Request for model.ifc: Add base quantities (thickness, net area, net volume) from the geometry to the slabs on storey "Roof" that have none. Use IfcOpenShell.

First a look at what the model holds.

```python
import ifcopenshell
import ifcopenshell.util.element
import ifcopenshell.util.unit

model = ifcopenshell.open("model.ifc")
print(model.schema)
for unit_type in ("LENGTHUNIT", "AREAUNIT", "VOLUMEUNIT"):
    print(unit_type, ifcopenshell.util.unit.calculate_unit_scale(model, unit_type))
storey = next(s for s in model.by_type("IfcBuildingStorey") if s.Name == "Roof")
slabs = [e for e in ifcopenshell.util.element.get_decomposition(storey) if e.is_a("IfcSlab")]
for e in sorted(slabs, key=lambda e: e.id()):
    print(e.id(), e.is_a(), e.Name, list(ifcopenshell.util.element.get_psets(e, qtos_only=True)), sep=" | ")
```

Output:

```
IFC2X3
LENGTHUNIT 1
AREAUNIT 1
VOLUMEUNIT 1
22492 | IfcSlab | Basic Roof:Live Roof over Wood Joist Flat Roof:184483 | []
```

```python
import ifcopenshell
import ifcopenshell.api.pset
import ifcopenshell.geom
import ifcopenshell.util.element
import ifcopenshell.util.shape
import ifcopenshell.util.unit

model = ifcopenshell.open("model.ifc")
unit_scale = ifcopenshell.util.unit.calculate_unit_scale(model)
area_scale = ifcopenshell.util.unit.calculate_unit_scale(model, "AREAUNIT")
volume_scale = ifcopenshell.util.unit.calculate_unit_scale(model, "VOLUMEUNIT")
settings = ifcopenshell.geom.settings()

storey = next(s for s in model.by_type("IfcBuildingStorey") if s.Name == "Roof")
slabs = [e for e in ifcopenshell.util.element.get_decomposition(storey) if e.is_a("IfcSlab")]

for e in sorted(slabs, key=lambda e: e.id()):
    if ifcopenshell.util.element.get_psets(e, qtos_only=True, should_inherit=False):
        continue
    # Geometry comes back in metres, in the element's own axes.
    shape = ifcopenshell.geom.create_shape(settings, e)
    values = {
        "Width": ifcopenshell.util.shape.get_z(shape.geometry) / unit_scale,
        "NetArea": ifcopenshell.util.shape.get_footprint_area(shape.geometry) / area_scale,
        "NetVolume": ifcopenshell.util.shape.get_volume(shape.geometry) / volume_scale,
    }
    qto = ifcopenshell.api.pset.add_qto(model, product=e, name="BaseQuantities")
    ifcopenshell.api.pset.edit_qto(model, qto=qto, properties=values)
    print(e.id(), {k: round(v, 3) for k, v in values.items()})

model.write("model_updated.ifc")
```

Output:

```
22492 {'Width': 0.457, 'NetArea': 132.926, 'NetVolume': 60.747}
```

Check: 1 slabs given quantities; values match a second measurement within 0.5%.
